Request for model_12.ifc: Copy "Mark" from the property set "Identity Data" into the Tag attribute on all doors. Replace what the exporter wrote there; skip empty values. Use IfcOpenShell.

First a look at what the model holds.

```python
import ifcopenshell
import ifcopenshell.util.element

model = ifcopenshell.open("model_12.ifc")
print(model.schema)
doors = model.by_type("IfcDoor")
print(len(doors), "doors")
for e in doors[:8]:
    source = ifcopenshell.util.element.get_pset(e, "Identity Data", "Mark")
    target = e.Tag
    print(e.id(), repr(source), repr(target), sep=" | ")
```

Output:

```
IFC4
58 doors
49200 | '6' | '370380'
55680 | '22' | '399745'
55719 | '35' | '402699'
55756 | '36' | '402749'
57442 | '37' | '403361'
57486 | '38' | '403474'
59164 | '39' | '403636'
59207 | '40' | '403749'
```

```python
import ifcopenshell
import ifcopenshell.util.element

model = ifcopenshell.open("model_12.ifc")

count = 0
for e in model.by_type("IfcDoor"):
    value = ifcopenshell.util.element.get_pset(e, "Identity Data", "Mark")
    current = e.Tag
    if not value or not value.strip() or current == value:
        continue
    e.Tag = value
    count += 1

print(count, "doors updated")

model.write("model_12_v2.ifc")
```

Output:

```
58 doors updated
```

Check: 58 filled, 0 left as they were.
